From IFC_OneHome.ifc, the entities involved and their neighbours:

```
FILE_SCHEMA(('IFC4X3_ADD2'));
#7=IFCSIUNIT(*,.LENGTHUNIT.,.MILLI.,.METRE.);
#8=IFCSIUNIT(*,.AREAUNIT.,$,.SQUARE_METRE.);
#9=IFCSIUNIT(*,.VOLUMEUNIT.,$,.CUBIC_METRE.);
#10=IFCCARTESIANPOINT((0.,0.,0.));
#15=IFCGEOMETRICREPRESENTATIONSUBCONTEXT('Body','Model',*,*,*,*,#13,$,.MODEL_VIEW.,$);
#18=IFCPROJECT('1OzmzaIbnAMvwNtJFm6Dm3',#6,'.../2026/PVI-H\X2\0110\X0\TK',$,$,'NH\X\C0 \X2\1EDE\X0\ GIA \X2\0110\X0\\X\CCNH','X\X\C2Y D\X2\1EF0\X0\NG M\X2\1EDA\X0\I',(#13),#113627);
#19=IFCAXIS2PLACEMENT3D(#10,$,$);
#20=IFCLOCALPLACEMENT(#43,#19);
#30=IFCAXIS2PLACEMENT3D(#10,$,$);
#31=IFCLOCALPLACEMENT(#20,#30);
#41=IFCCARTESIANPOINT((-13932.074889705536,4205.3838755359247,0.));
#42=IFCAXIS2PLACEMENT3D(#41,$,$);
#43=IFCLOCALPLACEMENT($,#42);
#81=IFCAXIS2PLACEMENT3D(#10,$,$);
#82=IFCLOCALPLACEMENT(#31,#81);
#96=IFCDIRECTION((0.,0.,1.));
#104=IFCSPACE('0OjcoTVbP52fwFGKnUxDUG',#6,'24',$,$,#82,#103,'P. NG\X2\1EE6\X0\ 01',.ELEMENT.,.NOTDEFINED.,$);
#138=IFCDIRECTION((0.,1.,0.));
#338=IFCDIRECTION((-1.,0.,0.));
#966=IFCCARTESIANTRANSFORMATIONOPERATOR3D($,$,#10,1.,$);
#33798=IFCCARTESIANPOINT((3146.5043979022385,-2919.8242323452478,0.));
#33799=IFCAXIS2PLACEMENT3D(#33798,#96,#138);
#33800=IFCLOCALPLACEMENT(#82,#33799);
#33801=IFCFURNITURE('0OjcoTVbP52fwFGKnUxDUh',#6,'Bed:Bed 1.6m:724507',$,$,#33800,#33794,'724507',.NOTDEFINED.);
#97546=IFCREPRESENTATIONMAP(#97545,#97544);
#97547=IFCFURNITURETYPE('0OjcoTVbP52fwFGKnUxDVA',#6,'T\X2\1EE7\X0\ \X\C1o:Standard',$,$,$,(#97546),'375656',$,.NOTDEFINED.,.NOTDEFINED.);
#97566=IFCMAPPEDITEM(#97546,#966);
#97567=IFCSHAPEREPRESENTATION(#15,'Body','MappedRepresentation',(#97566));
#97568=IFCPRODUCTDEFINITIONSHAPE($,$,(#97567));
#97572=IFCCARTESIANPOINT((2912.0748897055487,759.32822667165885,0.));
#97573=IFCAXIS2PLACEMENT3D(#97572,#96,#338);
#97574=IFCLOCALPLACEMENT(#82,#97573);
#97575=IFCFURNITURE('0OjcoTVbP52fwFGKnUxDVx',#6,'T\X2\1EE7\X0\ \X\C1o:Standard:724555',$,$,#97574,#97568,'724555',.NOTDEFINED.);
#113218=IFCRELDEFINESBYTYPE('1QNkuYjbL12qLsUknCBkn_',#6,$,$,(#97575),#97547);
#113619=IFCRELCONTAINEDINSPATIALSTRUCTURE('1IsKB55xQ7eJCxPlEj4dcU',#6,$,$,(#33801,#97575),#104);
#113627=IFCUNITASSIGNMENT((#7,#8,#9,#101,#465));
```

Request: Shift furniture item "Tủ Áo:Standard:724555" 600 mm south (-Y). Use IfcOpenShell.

```python
import ifcopenshell
import ifcopenshell.api.geometry
import ifcopenshell.util.placement
import ifcopenshell.util.unit

model = ifcopenshell.open("IFC_OneHome.ifc")
unit_scale = ifcopenshell.util.unit.calculate_unit_scale(model)

item = model.by_guid("0OjcoTVbP52fwFGKnUxDVx")
matrix = ifcopenshell.util.placement.get_local_placement(item.ObjectPlacement)
matrix[1, 3] -= 0.6 / unit_scale
ifcopenshell.api.geometry.edit_object_placement(model, product=item, matrix=matrix, is_si=False)

print(ifcopenshell.util.placement.get_local_placement(item.ObjectPlacement).round(3) + 0.0)

model.write("IFC_OneHome-out.ifc")
```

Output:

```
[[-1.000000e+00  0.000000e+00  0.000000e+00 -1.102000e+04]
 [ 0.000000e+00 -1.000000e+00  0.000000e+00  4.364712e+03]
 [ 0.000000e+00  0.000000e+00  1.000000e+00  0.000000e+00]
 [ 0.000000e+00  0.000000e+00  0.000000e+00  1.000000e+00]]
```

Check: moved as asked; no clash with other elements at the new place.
